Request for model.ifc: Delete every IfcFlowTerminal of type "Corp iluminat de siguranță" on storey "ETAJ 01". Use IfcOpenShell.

First a look at what the model holds.

```python
import ifcopenshell
import ifcopenshell.util.element

model = ifcopenshell.open("model.ifc")
print(model.schema)
storey = next(s for s in model.by_type("IfcBuildingStorey") if s.Name == "ETAJ 01")
terminals = [e for e in ifcopenshell.util.element.get_decomposition(storey) if e.is_a("IfcFlowTerminal")]
seen = {}
for e in terminals:
    element_type = ifcopenshell.util.element.get_type(e)
    name = element_type.Name if element_type not in (None, e) else None
    seen[name] = seen.get(name, 0) + 1
for name, count in sorted(seen.items(), key=str):
    print(count, "x", name)
```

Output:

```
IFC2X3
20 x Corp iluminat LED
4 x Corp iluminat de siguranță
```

```python
import ifcopenshell
import ifcopenshell.api.root
import ifcopenshell.util.element

model = ifcopenshell.open("model.ifc")

storey = next(s for s in model.by_type("IfcBuildingStorey") if s.Name == "ETAJ 01")
terminals = [e for e in ifcopenshell.util.element.get_decomposition(storey) if e.is_a("IfcFlowTerminal")]
targets = [e for e in terminals if (t := ifcopenshell.util.element.get_type(e)) not in (None, e) and t.Name == "Corp iluminat de siguranță"]

for e in targets:
    ifcopenshell.api.root.remove_product(model, product=e)
print(len(targets), "removed")

model.write("model_updated.ifc")
```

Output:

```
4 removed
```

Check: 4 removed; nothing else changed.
